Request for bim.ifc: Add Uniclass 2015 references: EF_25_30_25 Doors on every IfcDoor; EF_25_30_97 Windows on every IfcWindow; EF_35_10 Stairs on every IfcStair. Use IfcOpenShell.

First a look at what the model holds.

```python
import ifcopenshell

model = ifcopenshell.open("bim.ifc")
print(model.schema)
print("classifications:", [c.Name for c in model.by_type("IfcClassification")])
for ifc_class in ("IfcDoor", "IfcRoof", "IfcStair", "IfcWall", "IfcWindow"):
    print(ifc_class, len(model.by_type(ifc_class)))
```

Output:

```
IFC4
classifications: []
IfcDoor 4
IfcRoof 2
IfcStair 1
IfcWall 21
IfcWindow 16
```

```python
import ifcopenshell
import ifcopenshell.api.classification

model = ifcopenshell.open("bim.ifc")

system = ifcopenshell.api.classification.add_classification(model, classification="Uniclass 2015")

codes = {
    "IfcDoor": ("EF_25_30_25", "Doors"),
    "IfcWindow": ("EF_25_30_97", "Windows"),
    "IfcStair": ("EF_35_10", "Stairs"),
}
for ifc_class, (code, name) in codes.items():
    products = model.by_type(ifc_class)
    ifcopenshell.api.classification.add_reference(
        model, products=products, classification=system, identification=code, name=name
    )
    print(code, len(products))

model.write("bim_v2.ifc")
```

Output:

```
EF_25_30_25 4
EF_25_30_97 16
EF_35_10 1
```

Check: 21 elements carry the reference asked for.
